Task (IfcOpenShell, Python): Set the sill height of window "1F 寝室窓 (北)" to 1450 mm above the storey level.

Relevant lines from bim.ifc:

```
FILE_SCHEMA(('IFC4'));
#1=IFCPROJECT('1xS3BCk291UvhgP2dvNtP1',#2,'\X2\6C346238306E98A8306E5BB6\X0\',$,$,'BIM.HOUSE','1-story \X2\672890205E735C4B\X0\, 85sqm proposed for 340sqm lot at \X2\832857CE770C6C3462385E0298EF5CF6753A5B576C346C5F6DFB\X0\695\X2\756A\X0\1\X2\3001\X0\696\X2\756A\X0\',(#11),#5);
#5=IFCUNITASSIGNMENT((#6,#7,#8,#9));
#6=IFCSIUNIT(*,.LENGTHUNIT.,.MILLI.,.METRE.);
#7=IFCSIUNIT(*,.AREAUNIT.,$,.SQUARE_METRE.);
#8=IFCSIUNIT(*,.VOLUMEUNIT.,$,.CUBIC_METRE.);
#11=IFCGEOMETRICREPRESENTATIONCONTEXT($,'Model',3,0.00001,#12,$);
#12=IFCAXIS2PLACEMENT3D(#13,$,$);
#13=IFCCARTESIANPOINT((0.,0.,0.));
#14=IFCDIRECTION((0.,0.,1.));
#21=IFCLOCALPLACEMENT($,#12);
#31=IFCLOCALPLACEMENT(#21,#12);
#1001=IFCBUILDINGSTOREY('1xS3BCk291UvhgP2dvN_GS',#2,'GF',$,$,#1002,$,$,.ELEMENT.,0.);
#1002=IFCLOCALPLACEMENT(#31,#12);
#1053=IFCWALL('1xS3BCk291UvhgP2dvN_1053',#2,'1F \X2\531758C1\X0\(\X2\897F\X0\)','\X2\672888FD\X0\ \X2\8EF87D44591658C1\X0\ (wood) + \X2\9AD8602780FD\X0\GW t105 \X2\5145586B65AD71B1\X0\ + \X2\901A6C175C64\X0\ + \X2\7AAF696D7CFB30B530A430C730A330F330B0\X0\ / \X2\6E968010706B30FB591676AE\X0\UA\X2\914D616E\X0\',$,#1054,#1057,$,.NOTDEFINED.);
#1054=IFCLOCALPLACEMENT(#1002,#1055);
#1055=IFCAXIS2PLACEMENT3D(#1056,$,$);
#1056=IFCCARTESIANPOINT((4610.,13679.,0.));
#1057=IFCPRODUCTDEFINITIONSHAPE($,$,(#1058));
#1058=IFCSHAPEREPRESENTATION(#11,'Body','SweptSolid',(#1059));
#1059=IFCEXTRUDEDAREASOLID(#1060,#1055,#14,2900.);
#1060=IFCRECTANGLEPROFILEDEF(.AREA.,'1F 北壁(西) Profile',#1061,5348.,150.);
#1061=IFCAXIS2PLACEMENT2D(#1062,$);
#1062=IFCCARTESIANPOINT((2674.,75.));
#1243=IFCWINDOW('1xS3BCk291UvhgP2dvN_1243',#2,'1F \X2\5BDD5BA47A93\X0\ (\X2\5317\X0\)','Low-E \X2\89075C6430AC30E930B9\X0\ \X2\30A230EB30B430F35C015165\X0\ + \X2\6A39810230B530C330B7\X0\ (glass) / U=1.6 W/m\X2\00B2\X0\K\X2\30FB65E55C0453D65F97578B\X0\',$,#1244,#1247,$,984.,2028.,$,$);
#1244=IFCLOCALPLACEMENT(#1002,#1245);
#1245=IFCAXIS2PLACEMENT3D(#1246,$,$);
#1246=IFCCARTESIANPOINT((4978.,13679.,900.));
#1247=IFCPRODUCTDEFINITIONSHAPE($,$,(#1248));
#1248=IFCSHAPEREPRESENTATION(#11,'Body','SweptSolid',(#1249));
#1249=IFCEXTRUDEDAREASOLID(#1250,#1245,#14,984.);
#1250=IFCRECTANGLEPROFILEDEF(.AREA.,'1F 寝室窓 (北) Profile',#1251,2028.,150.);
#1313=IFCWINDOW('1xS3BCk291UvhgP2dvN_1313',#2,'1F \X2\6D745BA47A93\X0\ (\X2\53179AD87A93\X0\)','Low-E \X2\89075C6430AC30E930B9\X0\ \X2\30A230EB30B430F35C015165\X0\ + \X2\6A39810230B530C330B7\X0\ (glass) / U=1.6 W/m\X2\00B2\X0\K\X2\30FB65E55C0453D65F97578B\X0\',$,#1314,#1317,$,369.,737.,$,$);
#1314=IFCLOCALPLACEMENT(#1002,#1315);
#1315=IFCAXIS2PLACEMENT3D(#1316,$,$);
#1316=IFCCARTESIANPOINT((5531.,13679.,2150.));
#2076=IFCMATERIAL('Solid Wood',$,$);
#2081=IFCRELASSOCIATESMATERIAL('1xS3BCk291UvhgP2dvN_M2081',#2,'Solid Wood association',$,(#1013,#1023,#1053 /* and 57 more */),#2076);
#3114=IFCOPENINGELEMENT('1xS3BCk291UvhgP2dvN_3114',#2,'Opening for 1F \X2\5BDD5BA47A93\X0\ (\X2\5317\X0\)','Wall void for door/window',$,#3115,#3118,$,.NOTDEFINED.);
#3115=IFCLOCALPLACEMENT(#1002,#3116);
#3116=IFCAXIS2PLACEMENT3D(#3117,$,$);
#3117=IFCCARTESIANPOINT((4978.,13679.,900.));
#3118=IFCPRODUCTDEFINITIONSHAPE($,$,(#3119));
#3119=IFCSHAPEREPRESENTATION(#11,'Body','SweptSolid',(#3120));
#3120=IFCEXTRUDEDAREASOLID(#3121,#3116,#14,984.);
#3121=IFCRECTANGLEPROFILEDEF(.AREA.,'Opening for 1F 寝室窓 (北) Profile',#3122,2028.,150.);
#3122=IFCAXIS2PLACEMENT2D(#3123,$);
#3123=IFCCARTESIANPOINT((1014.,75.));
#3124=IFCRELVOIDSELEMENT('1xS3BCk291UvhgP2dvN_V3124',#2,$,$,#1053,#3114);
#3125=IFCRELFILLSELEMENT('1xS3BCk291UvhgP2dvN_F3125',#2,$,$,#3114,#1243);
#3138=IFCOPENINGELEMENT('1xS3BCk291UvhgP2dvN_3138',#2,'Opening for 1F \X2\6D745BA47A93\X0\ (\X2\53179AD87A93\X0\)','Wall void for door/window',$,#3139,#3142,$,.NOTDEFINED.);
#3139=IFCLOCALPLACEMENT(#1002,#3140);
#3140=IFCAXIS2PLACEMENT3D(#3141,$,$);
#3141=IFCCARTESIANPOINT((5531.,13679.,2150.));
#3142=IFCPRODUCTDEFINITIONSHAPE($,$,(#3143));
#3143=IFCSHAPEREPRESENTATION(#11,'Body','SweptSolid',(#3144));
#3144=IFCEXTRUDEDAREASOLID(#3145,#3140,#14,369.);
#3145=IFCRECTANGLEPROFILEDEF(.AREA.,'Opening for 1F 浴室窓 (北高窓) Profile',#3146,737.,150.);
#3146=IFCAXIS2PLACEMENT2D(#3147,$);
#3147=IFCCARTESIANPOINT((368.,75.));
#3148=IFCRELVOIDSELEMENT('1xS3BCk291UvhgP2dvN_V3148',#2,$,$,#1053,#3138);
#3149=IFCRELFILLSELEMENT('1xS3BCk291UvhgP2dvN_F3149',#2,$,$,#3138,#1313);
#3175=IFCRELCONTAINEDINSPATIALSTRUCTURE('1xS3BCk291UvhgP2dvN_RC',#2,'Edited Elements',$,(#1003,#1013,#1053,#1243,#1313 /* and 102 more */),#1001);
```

```python
import numpy as np
import ifcopenshell
import ifcopenshell.api.geometry
import ifcopenshell.geom
import ifcopenshell.util.element
import ifcopenshell.util.placement
import ifcopenshell.util.shape
import ifcopenshell.util.unit

model = ifcopenshell.open("bim.ifc")
unit_scale = ifcopenshell.util.unit.calculate_unit_scale(model)

window = model.by_id(1243)
opening = window.FillsVoids[0].RelatingOpeningElement
storey = ifcopenshell.util.element.get_container(window, ifc_class="IfcBuildingStorey")
level = ifcopenshell.util.placement.get_local_placement(storey.ObjectPlacement)[2, 3]

# The opening's origin need not be at the sill, so measure its lowest point.
shape = ifcopenshell.geom.create_shape(ifcopenshell.geom.settings(), opening)
bottom = ifcopenshell.util.shape.get_shape_bottom_elevation(shape, shape.geometry) / unit_scale
dz = level + 1.45 / unit_scale - bottom

shift = np.array([0.0, 0.0, dz])
# The window is not placed relative to its opening, so move both.
for product in (opening, window):
    matrix = ifcopenshell.util.placement.get_local_placement(product.ObjectPlacement)
    matrix[:3, 3] += shift
    ifcopenshell.api.geometry.edit_object_placement(model, product=product, matrix=matrix, is_si=False)

print(f"moved by {dz * unit_scale:+.3f} m")

model.write("bim_v2.ifc")
```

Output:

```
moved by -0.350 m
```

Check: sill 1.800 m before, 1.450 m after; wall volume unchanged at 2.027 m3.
